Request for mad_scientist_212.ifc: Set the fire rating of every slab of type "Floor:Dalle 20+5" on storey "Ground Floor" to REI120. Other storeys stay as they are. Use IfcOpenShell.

First a look at what the model holds.

```python
import ifcopenshell
import ifcopenshell.util.element

model = ifcopenshell.open("mad_scientist_212.ifc")
print(model.schema)
storey = next(s for s in model.by_type("IfcBuildingStorey") if s.Name == "Ground Floor")
slabs = [e for e in ifcopenshell.util.element.get_decomposition(storey) if e.is_a("IfcSlab")]
seen = {}
for e in slabs:
    element_type = ifcopenshell.util.element.get_type(e)
    key = (element_type.Name if element_type != e and element_type else None, ifcopenshell.util.element.get_pset(e, "Pset_SlabCommon", "FireRating"))
    seen[key] = seen.get(key, 0) + 1
for (name, value), count in sorted(seen.items(), key=str):
    print(count, "x", name, "|", value)
```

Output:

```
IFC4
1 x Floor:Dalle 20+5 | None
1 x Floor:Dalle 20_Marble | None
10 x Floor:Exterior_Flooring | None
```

```python
import ifcopenshell
import ifcopenshell.api.pset
import ifcopenshell.util.element

model = ifcopenshell.open("mad_scientist_212.ifc")

storey = next(s for s in model.by_type("IfcBuildingStorey") if s.Name == "Ground Floor")
slabs = [e for e in ifcopenshell.util.element.get_decomposition(storey) if e.is_a("IfcSlab")]

count = 0
for e in slabs:
    element_type = ifcopenshell.util.element.get_type(e)
    if element_type in (None, e) or element_type.Name != "Floor:Dalle 20+5":
        continue
    # add_pset returns the element's existing set when there is one.
    pset = ifcopenshell.api.pset.add_pset(model, product=e, name="Pset_SlabCommon")
    ifcopenshell.api.pset.edit_pset(model, pset=pset, properties={"FireRating": "REI120"})
    count += 1

print(count, "slabs updated")

model.write("mad_scientist_212-out.ifc")
```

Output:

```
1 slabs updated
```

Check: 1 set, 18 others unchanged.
